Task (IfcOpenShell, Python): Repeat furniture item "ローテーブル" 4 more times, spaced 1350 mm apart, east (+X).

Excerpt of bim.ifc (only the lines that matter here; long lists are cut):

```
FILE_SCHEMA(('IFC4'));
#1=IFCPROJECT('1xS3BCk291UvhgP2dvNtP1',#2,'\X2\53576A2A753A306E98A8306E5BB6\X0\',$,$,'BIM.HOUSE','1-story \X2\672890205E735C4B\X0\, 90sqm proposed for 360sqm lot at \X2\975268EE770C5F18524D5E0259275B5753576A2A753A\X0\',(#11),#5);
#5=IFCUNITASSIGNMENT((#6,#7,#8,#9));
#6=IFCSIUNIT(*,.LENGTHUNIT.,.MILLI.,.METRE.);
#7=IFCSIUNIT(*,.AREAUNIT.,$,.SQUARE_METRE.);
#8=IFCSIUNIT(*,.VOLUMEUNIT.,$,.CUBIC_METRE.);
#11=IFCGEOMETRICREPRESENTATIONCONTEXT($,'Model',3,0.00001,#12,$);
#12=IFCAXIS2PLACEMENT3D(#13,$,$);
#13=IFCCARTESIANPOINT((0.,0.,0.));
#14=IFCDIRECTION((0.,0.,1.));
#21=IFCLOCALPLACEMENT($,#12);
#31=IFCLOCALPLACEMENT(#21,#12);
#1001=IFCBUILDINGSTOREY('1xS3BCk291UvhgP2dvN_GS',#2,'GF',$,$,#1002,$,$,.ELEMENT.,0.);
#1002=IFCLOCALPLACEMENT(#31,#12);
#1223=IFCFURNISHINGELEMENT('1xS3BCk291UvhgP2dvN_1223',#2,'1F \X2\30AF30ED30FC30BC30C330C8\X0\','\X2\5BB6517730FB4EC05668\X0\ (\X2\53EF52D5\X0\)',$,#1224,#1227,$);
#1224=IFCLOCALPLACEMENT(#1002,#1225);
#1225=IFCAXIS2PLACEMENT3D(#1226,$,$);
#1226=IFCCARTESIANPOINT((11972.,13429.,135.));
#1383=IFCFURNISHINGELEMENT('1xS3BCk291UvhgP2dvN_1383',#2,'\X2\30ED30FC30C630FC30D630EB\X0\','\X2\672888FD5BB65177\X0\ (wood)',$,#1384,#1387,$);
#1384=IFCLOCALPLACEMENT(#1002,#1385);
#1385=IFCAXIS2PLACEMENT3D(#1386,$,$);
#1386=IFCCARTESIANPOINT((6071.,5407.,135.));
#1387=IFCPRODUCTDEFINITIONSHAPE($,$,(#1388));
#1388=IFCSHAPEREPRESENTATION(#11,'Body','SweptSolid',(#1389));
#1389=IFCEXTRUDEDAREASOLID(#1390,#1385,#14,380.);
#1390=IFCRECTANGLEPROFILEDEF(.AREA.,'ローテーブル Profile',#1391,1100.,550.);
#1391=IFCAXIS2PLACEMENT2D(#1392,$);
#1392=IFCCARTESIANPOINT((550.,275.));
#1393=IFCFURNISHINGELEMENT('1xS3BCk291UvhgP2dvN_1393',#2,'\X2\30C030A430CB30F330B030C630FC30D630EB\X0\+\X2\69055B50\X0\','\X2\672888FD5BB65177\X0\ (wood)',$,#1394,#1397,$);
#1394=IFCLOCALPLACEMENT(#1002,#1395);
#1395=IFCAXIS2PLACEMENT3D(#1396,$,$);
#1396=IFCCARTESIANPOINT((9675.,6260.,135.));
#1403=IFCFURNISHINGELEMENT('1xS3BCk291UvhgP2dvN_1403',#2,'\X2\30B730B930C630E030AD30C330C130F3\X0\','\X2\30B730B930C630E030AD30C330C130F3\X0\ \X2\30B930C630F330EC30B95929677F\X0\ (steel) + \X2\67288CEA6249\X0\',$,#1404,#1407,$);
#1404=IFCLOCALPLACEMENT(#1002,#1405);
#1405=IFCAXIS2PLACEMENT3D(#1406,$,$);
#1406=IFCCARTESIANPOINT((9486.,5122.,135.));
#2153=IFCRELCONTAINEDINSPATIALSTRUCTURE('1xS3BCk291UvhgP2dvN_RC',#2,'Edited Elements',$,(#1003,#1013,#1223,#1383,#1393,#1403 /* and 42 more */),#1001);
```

```python
import numpy as np
import ifcopenshell
import ifcopenshell.api.geometry
import ifcopenshell.api.root
import ifcopenshell.util.element
import ifcopenshell.util.placement

model = ifcopenshell.open("bim.ifc")


def reuse_history(source, copy):
    """copy_class also copies each property set's owner history, people and application; keep the originals."""
    for rel in copy.IsDefinedBy:
        if rel.is_a("IfcRelDefinesByProperties") and (history := rel.RelatingPropertyDefinition.OwnerHistory):
            rel.RelatingPropertyDefinition.OwnerHistory = source.OwnerHistory
            ifcopenshell.util.element.remove_deep2(model, history)


source = model.by_guid("1xS3BCk291UvhgP2dvN_1383")
base = ifcopenshell.util.placement.get_local_placement(source.ObjectPlacement)
step = np.array([1.0, 0.0, 0.0]) * 1350.0

for i in range(1, 5):
    copy = ifcopenshell.api.root.copy_class(model, product=source)
    copy.Representation = ifcopenshell.util.element.copy_deep(
        model, source.Representation, exclude=["IfcGeometricRepresentationContext", "IfcRepresentationMap"]
    )
    reuse_history(source, copy)
    matrix = base.copy()
    matrix[:3, 3] += i * step
    print("added at", matrix[:3, 3].round(3) + 0.0)
    ifcopenshell.api.geometry.edit_object_placement(model, product=copy, matrix=matrix, is_si=False)

model.write("bim_v2.ifc")
```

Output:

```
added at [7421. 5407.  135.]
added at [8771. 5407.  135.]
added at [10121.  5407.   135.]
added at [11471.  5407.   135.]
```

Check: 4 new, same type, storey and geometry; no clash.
